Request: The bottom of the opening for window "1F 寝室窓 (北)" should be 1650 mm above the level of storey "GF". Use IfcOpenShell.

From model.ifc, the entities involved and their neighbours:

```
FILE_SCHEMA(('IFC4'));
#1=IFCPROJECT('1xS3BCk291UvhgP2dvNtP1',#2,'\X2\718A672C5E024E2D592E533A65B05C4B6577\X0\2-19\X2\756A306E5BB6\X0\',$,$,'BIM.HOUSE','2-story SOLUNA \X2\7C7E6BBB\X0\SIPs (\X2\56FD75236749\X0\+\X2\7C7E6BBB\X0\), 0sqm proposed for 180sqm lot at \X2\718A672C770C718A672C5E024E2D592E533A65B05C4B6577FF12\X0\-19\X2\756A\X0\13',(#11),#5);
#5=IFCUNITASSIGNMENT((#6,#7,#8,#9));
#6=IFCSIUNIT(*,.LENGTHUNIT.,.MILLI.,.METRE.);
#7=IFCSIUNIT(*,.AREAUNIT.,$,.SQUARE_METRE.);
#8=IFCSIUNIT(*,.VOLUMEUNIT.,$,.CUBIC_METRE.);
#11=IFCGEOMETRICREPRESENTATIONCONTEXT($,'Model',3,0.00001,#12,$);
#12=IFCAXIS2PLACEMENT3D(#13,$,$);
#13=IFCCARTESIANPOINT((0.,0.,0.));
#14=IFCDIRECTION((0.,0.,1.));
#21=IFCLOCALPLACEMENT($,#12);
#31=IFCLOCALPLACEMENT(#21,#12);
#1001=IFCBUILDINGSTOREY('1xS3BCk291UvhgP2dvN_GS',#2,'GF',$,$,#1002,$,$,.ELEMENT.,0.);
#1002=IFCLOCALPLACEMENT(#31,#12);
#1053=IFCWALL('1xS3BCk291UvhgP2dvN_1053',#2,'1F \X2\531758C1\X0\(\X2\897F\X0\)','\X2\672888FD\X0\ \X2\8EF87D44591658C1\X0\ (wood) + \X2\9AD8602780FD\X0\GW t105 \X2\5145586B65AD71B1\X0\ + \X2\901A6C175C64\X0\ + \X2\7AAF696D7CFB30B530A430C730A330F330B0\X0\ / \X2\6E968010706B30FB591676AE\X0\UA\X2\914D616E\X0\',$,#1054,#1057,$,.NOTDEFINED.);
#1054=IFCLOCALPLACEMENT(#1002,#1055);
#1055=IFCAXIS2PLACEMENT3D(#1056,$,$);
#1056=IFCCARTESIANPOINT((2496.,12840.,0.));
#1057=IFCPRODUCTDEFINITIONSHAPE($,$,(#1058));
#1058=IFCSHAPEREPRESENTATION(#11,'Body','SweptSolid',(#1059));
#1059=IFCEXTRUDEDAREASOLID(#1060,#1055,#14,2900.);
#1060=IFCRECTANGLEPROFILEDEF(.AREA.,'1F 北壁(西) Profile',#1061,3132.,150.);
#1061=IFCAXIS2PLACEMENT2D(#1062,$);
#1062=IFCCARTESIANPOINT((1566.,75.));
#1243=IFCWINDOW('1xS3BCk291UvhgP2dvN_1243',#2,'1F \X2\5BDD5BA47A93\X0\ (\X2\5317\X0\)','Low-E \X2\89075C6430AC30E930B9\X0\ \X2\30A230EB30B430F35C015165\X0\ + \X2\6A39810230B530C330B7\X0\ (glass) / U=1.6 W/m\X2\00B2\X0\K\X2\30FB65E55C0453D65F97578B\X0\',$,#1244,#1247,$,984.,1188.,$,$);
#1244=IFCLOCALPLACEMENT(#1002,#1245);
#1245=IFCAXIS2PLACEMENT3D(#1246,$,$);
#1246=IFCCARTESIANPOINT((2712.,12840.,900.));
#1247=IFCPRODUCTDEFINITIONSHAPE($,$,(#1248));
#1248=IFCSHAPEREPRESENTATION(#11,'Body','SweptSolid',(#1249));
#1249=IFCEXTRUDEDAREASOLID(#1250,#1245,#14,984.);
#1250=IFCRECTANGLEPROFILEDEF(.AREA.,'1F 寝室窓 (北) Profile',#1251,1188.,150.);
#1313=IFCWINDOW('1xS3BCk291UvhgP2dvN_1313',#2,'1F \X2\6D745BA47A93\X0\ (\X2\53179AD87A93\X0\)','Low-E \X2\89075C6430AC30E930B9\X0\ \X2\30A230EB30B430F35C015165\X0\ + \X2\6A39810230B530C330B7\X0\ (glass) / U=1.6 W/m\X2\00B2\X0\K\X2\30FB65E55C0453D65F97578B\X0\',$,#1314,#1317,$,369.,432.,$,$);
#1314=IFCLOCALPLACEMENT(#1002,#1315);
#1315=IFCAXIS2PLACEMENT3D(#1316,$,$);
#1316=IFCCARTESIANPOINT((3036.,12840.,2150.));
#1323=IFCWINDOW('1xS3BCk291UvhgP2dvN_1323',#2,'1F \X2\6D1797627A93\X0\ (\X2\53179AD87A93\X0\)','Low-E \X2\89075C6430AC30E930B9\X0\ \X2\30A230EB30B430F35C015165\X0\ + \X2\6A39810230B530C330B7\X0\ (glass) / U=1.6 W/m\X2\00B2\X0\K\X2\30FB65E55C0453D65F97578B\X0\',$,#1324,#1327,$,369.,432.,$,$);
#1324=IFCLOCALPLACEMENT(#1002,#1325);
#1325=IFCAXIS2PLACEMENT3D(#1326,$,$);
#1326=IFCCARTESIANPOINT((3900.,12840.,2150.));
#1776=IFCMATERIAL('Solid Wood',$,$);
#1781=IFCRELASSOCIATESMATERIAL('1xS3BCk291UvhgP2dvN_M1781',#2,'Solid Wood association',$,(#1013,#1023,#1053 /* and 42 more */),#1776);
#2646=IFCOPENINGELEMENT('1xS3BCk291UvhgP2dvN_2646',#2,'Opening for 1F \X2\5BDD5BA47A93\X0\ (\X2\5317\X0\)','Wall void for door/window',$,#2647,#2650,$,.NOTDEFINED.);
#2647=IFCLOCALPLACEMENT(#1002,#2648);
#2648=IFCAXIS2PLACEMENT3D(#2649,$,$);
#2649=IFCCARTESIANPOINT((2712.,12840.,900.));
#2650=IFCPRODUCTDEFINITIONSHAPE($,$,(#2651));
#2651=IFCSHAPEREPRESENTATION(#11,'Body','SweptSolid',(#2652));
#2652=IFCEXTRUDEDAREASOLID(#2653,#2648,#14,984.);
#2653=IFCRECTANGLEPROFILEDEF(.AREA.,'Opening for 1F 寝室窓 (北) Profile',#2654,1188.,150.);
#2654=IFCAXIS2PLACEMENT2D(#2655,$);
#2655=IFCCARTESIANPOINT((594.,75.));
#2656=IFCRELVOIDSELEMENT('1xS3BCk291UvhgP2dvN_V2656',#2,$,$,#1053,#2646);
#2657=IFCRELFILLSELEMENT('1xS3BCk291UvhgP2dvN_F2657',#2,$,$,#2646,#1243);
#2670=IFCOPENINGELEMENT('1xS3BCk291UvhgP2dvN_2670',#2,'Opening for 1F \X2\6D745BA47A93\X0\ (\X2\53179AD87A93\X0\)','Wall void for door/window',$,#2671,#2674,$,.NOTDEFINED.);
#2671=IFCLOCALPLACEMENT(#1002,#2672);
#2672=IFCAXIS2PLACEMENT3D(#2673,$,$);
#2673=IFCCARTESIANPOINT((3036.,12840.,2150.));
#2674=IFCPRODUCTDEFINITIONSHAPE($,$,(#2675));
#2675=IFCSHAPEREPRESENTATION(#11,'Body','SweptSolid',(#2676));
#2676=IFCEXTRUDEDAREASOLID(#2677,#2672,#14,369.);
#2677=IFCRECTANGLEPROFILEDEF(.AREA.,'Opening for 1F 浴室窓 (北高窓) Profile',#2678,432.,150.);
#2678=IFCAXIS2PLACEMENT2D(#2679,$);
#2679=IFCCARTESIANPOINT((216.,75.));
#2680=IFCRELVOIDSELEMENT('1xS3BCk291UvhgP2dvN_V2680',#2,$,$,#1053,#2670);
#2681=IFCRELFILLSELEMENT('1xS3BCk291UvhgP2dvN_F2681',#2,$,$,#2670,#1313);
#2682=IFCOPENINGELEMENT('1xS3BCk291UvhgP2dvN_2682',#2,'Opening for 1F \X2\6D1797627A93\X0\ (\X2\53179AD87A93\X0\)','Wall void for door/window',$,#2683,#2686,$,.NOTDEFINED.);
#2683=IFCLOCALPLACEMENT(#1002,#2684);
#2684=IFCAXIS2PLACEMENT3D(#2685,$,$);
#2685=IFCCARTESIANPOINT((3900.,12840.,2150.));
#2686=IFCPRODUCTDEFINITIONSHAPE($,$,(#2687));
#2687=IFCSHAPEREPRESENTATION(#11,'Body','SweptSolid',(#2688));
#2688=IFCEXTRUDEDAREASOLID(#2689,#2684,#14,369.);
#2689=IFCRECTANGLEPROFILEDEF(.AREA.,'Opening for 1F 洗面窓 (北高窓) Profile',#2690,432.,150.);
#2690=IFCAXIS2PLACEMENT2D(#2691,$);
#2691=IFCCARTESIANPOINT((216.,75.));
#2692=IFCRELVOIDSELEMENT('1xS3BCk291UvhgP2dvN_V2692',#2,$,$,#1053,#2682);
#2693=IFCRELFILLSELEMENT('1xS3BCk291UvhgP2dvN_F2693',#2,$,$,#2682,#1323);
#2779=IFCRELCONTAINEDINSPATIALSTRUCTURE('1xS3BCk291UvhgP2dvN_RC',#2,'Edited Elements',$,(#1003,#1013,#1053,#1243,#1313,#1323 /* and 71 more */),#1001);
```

```python
import numpy as np
import ifcopenshell
import ifcopenshell.api.geometry
import ifcopenshell.geom
import ifcopenshell.util.element
import ifcopenshell.util.placement
import ifcopenshell.util.shape
import ifcopenshell.util.unit

model = ifcopenshell.open("model.ifc")
unit_scale = ifcopenshell.util.unit.calculate_unit_scale(model)

window = model.by_guid("1xS3BCk291UvhgP2dvN_1243")
opening = window.FillsVoids[0].RelatingOpeningElement
storey = ifcopenshell.util.element.get_container(window, ifc_class="IfcBuildingStorey")
level = ifcopenshell.util.placement.get_local_placement(storey.ObjectPlacement)[2, 3]

# The opening's origin need not be at the sill, so measure its lowest point.
shape = ifcopenshell.geom.create_shape(ifcopenshell.geom.settings(), opening)
bottom = ifcopenshell.util.shape.get_shape_bottom_elevation(shape, shape.geometry) / unit_scale
dz = level + 1.65 / unit_scale - bottom

shift = np.array([0.0, 0.0, dz])
# The window is not placed relative to its opening, so move both.
for product in (opening, window):
    matrix = ifcopenshell.util.placement.get_local_placement(product.ObjectPlacement)
    matrix[:3, 3] += shift
    ifcopenshell.api.geometry.edit_object_placement(model, product=product, matrix=matrix, is_si=False)

print(f"moved by {dz * unit_scale:+.3f} m")

model.write("model-out.ifc")
```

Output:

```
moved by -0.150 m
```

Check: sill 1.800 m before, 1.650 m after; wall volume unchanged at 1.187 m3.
